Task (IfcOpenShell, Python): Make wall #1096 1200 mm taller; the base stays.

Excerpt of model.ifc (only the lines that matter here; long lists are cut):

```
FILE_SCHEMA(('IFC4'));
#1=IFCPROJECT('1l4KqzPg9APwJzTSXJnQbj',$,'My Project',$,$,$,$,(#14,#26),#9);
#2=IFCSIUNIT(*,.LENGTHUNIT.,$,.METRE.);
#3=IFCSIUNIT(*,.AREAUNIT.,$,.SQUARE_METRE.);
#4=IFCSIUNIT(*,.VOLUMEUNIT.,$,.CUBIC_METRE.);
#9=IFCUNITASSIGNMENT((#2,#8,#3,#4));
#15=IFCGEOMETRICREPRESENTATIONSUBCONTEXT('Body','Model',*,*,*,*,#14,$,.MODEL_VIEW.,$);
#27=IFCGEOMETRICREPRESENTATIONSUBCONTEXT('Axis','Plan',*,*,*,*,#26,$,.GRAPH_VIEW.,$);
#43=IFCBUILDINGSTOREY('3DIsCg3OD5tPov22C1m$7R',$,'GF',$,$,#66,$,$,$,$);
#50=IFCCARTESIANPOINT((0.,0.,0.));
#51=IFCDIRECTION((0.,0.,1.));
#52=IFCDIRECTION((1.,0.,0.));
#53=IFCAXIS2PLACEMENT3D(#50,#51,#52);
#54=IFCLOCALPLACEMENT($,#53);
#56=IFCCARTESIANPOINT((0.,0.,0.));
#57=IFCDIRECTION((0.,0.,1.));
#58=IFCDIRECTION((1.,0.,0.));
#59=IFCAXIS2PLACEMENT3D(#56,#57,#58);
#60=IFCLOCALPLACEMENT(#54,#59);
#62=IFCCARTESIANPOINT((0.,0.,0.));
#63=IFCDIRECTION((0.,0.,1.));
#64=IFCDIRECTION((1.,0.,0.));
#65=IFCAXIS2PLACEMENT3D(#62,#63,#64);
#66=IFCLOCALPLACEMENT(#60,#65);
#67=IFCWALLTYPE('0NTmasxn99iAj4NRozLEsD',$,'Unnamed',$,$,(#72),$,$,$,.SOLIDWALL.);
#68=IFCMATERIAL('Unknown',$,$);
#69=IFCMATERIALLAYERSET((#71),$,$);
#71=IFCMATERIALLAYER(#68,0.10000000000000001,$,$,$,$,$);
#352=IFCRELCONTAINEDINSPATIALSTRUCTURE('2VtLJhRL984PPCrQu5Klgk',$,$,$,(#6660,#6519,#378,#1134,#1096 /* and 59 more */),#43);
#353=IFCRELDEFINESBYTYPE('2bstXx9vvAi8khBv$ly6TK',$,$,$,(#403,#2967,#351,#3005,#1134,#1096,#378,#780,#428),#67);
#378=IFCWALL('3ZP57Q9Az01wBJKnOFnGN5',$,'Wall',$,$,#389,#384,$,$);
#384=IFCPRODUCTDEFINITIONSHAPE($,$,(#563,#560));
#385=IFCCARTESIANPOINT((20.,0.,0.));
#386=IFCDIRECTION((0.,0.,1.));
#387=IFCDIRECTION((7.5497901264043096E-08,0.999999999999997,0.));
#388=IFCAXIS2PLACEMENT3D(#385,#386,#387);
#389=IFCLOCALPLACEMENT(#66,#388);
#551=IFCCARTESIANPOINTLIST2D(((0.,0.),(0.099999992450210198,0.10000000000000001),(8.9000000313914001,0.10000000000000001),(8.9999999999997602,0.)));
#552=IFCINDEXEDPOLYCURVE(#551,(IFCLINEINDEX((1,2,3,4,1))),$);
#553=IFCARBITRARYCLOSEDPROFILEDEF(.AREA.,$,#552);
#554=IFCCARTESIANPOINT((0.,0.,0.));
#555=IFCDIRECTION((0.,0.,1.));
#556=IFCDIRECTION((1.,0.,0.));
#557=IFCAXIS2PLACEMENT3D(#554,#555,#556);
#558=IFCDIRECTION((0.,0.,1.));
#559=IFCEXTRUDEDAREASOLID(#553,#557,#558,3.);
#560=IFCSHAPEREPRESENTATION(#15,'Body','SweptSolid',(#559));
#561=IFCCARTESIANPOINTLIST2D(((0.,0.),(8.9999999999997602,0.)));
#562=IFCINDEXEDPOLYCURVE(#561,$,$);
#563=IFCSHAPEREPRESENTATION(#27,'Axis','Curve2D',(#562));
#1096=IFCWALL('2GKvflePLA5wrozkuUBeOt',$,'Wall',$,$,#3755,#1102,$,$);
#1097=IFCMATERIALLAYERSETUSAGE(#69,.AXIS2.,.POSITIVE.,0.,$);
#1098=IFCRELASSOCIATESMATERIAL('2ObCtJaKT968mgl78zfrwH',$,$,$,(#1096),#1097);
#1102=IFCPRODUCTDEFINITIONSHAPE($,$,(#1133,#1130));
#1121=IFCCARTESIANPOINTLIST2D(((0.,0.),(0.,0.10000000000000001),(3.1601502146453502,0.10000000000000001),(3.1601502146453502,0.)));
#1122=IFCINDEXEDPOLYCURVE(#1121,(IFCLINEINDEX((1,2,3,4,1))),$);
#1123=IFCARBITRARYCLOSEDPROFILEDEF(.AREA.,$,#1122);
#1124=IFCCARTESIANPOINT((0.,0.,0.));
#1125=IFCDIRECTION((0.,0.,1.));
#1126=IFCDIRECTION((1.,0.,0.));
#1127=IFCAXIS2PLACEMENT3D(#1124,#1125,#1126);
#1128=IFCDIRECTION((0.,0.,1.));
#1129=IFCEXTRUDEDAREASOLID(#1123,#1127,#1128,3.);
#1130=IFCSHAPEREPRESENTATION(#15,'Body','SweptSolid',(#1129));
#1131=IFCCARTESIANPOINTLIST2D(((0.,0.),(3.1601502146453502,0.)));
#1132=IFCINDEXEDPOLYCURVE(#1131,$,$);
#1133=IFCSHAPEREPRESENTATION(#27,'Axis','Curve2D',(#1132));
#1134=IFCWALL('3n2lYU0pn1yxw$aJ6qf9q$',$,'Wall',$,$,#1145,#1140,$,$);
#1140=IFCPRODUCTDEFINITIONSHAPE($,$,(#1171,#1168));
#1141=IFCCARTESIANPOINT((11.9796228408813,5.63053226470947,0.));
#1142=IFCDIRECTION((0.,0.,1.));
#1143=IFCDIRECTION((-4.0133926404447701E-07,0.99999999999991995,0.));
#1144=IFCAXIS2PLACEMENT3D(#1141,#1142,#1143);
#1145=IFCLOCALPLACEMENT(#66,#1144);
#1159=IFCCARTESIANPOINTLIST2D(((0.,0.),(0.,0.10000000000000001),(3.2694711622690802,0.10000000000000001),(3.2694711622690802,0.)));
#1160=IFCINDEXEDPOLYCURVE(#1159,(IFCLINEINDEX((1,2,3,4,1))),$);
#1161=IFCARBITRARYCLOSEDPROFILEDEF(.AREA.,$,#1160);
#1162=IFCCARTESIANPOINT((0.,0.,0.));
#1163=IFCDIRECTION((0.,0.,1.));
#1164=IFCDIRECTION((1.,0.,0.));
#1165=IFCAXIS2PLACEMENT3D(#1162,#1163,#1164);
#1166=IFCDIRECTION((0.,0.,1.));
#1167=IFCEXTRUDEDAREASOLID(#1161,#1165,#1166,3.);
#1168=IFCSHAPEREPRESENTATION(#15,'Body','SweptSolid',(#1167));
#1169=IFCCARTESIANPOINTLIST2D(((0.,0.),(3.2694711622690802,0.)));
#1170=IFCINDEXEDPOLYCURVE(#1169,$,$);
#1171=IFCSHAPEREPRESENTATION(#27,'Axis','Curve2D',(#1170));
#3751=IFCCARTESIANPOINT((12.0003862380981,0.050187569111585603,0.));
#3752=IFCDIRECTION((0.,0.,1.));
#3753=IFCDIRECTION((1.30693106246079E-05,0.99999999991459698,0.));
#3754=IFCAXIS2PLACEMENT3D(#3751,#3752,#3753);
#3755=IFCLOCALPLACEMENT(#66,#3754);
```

```python
import ifcopenshell
import ifcopenshell.geom
import ifcopenshell.util.representation
import ifcopenshell.util.shape
import ifcopenshell.util.unit

model = ifcopenshell.open("model.ifc")
unit_scale = ifcopenshell.util.unit.calculate_unit_scale(model)
settings = ifcopenshell.geom.settings()


def volume(element):
    """Net volume in cubic metres, openings subtracted."""
    shape = ifcopenshell.geom.create_shape(settings, element)
    return ifcopenshell.util.shape.get_volume(shape.geometry)


wall = model.by_id(1096)
before = volume(wall)

body = ifcopenshell.util.representation.get_representation(wall, "Model", "Body")
solid = body.Items[0]
old_height = solid.Depth
solid.Depth += 1.2 / unit_scale
after = volume(wall)

print(f"height {old_height:g} -> {solid.Depth:g}, volume {before:.3f} -> {after:.3f} m3")

model.write("model-out.ifc")
```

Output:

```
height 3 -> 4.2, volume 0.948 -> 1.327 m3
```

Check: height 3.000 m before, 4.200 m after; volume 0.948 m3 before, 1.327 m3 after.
